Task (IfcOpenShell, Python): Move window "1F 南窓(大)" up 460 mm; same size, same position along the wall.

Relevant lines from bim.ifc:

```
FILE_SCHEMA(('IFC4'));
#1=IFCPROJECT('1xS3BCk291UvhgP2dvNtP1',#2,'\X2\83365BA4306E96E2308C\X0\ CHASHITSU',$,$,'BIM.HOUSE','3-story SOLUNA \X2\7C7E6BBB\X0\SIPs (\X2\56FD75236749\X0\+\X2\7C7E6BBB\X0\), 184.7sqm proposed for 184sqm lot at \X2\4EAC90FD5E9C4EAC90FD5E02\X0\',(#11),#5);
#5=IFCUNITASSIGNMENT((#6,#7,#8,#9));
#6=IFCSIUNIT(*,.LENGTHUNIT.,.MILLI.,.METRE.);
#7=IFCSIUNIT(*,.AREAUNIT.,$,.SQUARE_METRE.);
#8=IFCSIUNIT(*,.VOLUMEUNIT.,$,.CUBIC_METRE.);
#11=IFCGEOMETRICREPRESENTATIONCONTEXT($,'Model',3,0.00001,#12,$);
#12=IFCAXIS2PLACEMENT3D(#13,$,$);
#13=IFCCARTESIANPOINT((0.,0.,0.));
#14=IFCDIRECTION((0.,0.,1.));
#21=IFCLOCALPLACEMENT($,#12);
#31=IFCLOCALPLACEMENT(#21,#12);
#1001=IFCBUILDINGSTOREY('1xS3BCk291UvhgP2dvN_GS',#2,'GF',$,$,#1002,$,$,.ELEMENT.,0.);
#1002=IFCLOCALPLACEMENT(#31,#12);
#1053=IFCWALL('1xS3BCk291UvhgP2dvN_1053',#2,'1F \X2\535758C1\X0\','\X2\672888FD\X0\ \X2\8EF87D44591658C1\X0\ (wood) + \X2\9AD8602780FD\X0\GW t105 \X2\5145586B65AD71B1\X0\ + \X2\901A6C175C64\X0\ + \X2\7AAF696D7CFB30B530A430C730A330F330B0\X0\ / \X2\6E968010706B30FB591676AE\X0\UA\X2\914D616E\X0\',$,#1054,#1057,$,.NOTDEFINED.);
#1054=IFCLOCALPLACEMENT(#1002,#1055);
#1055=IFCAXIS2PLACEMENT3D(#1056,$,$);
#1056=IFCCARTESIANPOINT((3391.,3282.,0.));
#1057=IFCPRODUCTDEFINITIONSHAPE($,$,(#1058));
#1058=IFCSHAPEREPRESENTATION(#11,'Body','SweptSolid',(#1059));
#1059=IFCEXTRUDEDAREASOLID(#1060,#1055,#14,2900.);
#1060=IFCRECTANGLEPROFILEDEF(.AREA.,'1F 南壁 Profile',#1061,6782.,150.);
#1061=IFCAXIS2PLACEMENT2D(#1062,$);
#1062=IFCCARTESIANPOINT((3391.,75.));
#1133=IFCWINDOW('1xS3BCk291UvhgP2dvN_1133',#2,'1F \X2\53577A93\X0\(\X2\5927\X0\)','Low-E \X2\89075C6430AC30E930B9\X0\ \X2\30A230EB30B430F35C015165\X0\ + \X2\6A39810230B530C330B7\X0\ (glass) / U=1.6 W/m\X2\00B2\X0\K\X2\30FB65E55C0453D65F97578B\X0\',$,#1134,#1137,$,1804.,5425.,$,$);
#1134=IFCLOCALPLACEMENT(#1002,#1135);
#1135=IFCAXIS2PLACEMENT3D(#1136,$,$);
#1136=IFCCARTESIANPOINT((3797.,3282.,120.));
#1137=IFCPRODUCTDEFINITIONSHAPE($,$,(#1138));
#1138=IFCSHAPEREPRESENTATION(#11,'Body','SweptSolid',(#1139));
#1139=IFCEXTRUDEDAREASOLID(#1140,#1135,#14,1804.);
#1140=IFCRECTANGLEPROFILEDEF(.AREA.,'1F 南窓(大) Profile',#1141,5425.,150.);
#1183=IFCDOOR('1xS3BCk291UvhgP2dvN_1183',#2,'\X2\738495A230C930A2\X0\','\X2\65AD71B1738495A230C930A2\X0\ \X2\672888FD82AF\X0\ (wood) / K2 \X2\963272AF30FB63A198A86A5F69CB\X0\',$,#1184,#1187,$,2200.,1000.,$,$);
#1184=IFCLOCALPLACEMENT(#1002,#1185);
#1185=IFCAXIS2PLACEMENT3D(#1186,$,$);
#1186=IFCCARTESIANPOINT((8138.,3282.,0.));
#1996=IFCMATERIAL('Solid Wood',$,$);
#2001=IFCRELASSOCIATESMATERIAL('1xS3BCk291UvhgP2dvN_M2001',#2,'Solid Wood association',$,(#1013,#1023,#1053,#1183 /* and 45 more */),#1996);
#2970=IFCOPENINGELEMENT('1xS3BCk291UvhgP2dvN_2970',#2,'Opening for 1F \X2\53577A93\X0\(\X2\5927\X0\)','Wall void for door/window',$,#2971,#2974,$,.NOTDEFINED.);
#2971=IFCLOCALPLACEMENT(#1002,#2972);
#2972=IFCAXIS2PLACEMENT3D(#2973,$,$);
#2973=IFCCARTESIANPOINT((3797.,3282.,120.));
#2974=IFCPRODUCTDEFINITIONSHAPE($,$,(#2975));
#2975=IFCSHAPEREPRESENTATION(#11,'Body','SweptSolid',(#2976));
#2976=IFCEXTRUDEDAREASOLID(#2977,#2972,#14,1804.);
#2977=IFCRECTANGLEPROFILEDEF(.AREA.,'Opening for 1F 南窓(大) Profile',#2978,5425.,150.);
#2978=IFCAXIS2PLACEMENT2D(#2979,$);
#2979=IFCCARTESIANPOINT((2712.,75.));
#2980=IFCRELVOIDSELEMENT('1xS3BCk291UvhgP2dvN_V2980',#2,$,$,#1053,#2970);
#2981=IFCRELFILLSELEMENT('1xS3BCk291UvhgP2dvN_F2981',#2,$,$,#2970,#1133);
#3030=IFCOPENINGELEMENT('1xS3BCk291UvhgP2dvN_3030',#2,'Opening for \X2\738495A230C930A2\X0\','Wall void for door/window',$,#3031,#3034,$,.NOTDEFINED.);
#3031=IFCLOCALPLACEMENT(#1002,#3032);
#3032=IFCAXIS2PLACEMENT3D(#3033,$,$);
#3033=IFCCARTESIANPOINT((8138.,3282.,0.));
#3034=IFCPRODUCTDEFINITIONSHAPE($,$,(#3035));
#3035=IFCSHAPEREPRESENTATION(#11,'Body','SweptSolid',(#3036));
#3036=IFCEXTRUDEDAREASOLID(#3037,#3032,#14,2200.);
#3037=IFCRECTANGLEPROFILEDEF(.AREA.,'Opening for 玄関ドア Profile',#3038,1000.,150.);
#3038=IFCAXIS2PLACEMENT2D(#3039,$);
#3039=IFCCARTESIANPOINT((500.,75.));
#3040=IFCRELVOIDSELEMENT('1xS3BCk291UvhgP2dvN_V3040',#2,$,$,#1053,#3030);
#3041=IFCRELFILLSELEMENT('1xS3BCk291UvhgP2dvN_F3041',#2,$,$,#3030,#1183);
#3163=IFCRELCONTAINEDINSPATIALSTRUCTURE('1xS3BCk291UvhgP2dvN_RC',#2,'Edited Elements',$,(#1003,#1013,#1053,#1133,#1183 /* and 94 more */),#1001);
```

```python
import numpy as np
import ifcopenshell
import ifcopenshell.api.geometry
import ifcopenshell.util.placement
import ifcopenshell.util.unit

model = ifcopenshell.open("bim.ifc")
unit_scale = ifcopenshell.util.unit.calculate_unit_scale(model)

window = model.by_guid("1xS3BCk291UvhgP2dvN_1133")
opening = window.FillsVoids[0].RelatingOpeningElement
dz = 460.0

shift = np.array([0.0, 0.0, dz])
# The window is not placed relative to its opening, so move both.
for product in (opening, window):
    matrix = ifcopenshell.util.placement.get_local_placement(product.ObjectPlacement)
    matrix[:3, 3] += shift
    ifcopenshell.api.geometry.edit_object_placement(model, product=product, matrix=matrix, is_si=False)

print(f"moved by {dz * unit_scale:+.3f} m")

model.write("bim_v2.ifc")
```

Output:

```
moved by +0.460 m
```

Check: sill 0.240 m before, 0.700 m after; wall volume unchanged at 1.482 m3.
